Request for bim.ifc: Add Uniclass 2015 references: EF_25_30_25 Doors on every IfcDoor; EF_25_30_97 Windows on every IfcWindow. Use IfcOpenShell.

First a look at what the model holds.

```python
import ifcopenshell

model = ifcopenshell.open("bim.ifc")
print(model.schema)
print("classifications:", [c.Name for c in model.by_type("IfcClassification")])
for ifc_class in ("IfcDoor", "IfcRoof", "IfcStair", "IfcWall", "IfcWindow"):
    print(ifc_class, len(model.by_type(ifc_class)))
```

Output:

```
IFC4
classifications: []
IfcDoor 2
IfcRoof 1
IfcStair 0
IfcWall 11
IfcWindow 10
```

```python
import ifcopenshell
import ifcopenshell.api.classification

model = ifcopenshell.open("bim.ifc")

system = ifcopenshell.api.classification.add_classification(model, classification="Uniclass 2015")

codes = {
    "IfcDoor": ("EF_25_30_25", "Doors"),
    "IfcWindow": ("EF_25_30_97", "Windows"),
}
for ifc_class, (code, name) in codes.items():
    products = model.by_type(ifc_class)
    ifcopenshell.api.classification.add_reference(
        model, products=products, classification=system, identification=code, name=name
    )
    print(code, len(products))

model.write("bim_rev.ifc")
```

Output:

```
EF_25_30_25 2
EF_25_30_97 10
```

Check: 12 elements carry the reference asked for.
